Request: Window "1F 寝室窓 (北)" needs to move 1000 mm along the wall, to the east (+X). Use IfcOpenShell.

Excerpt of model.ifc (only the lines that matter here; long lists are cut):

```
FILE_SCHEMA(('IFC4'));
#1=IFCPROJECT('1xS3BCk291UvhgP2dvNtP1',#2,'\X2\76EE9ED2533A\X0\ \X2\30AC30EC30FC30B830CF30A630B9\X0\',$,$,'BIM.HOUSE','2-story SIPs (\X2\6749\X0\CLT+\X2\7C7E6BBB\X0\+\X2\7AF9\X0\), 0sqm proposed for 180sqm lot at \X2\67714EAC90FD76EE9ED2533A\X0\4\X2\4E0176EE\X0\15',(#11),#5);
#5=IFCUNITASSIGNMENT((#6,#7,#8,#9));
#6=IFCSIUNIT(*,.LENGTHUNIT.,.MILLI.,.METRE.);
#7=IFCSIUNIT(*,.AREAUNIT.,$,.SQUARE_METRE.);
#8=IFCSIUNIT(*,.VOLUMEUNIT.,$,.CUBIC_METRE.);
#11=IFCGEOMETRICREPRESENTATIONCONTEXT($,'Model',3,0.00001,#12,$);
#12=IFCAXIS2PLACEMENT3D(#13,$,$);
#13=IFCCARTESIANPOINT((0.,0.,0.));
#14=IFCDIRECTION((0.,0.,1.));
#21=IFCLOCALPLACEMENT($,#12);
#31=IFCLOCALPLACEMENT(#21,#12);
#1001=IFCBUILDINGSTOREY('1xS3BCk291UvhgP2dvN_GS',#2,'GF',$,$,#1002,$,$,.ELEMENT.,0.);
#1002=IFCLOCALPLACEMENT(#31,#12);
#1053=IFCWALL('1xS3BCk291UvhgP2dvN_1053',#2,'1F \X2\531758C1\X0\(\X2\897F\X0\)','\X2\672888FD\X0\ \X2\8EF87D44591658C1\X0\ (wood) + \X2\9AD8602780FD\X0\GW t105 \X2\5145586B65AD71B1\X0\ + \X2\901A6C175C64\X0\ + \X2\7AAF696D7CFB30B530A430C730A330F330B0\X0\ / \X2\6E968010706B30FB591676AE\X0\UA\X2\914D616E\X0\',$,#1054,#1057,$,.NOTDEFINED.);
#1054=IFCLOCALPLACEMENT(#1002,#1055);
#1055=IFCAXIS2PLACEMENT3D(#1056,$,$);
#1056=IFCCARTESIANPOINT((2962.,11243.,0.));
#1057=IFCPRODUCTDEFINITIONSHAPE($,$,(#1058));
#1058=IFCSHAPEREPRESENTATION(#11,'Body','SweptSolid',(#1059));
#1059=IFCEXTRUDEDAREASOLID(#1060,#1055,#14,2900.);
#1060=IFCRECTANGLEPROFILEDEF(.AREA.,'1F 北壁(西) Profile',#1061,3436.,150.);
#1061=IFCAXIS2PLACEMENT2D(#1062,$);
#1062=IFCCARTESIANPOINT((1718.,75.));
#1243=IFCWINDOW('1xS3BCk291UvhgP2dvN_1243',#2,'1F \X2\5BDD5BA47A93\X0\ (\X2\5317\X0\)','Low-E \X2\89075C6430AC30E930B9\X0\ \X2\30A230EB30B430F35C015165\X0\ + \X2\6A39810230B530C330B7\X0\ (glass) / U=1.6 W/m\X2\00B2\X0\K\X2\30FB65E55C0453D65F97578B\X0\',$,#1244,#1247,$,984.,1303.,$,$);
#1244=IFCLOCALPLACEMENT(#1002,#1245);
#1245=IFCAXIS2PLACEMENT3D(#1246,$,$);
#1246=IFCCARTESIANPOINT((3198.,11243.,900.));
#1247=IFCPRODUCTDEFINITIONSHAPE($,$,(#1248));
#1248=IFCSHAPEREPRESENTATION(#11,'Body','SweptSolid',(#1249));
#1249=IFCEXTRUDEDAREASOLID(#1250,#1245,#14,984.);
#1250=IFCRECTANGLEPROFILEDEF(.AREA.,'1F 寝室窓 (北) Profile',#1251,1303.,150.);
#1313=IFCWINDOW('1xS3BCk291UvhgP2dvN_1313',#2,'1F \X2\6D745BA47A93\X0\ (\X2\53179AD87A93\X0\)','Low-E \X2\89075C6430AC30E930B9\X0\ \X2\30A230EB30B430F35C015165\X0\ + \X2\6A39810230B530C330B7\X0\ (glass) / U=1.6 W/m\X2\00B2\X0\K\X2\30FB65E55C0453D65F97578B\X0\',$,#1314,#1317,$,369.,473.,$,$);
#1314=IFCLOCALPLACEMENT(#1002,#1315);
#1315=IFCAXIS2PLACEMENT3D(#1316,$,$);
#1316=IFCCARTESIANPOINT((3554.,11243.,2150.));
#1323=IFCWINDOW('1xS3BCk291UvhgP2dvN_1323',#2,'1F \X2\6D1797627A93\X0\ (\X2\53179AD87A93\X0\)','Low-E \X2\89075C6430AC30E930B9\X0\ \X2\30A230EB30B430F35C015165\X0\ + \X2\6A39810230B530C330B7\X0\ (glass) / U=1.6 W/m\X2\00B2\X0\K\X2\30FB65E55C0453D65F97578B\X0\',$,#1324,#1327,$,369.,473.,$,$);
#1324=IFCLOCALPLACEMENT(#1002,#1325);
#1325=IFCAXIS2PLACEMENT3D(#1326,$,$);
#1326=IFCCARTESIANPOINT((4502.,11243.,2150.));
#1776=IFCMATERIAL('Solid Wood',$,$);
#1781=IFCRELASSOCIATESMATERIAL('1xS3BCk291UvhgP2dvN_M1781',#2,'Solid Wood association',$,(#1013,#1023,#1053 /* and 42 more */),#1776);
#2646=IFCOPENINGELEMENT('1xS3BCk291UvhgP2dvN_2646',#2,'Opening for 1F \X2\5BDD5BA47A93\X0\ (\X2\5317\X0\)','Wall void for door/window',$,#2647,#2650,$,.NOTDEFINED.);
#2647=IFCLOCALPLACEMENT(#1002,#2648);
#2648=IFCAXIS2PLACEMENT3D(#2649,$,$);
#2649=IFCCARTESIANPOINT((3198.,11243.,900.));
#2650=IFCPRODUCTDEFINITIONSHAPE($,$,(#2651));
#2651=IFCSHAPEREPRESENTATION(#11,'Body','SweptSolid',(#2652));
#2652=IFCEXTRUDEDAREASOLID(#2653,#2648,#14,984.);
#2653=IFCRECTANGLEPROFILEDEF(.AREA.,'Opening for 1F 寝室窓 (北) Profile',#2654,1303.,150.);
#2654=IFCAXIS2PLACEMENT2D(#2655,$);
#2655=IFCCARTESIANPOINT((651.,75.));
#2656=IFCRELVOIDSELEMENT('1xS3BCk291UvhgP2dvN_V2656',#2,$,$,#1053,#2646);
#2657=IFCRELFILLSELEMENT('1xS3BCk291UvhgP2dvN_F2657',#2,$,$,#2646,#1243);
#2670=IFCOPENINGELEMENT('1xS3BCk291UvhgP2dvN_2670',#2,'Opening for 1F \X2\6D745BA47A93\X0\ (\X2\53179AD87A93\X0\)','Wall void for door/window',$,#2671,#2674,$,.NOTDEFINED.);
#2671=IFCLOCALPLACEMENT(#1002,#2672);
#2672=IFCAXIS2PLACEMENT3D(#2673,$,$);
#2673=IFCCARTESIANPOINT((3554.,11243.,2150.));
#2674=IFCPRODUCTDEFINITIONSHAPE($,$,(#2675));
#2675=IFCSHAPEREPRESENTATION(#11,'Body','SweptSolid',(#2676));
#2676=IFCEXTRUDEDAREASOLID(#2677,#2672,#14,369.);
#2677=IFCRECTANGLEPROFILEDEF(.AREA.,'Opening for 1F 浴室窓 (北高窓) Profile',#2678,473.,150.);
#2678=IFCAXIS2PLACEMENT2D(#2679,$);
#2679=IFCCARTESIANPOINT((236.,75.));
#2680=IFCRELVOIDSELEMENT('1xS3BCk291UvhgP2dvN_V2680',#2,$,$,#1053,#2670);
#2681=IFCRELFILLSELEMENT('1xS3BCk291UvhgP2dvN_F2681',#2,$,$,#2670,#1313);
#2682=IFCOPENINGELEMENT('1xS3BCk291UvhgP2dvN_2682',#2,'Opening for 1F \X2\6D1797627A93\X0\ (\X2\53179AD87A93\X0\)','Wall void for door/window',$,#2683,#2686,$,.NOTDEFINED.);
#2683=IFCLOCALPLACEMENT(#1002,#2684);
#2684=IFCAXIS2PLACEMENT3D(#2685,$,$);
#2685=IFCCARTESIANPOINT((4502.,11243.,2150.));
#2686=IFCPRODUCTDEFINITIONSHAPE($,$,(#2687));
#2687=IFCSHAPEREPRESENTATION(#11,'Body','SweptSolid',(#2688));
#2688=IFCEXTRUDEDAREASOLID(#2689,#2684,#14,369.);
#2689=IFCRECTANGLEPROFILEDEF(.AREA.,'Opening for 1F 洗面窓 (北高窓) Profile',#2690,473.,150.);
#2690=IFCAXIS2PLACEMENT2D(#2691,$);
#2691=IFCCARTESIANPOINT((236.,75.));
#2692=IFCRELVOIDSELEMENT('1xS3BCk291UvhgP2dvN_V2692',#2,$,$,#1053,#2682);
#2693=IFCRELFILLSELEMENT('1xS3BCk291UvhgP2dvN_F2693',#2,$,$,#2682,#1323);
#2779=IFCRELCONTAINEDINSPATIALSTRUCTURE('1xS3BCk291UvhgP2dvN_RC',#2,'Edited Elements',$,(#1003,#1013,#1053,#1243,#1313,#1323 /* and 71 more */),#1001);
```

```python
import ifcopenshell
import ifcopenshell.api.geometry
import ifcopenshell.util.placement
import ifcopenshell.util.unit

model = ifcopenshell.open("model.ifc")
unit_scale = ifcopenshell.util.unit.calculate_unit_scale(model)

window = model.by_id(1243)
opening = window.FillsVoids[0].RelatingOpeningElement
wall = opening.VoidsElements[0].RelatingBuildingElement

wall_matrix = ifcopenshell.util.placement.get_local_placement(wall.ObjectPlacement)
shift = wall_matrix[:3, 0] * 1 / unit_scale
before = ifcopenshell.util.placement.get_local_placement(window.ObjectPlacement)[:3, 3].copy()

# The window is not placed relative to its opening, so move both.
for product in (opening, window):
    matrix = ifcopenshell.util.placement.get_local_placement(product.ObjectPlacement)
    matrix[:3, 3] += shift
    ifcopenshell.api.geometry.edit_object_placement(model, product=product, matrix=matrix, is_si=False)

after = ifcopenshell.util.placement.get_local_placement(window.ObjectPlacement)[:3, 3]
print("window moved by", (after - before).round(3) + 0.0)

model.write("model_v2.ifc")
```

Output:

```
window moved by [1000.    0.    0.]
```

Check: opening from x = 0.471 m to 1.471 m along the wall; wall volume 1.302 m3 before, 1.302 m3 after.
